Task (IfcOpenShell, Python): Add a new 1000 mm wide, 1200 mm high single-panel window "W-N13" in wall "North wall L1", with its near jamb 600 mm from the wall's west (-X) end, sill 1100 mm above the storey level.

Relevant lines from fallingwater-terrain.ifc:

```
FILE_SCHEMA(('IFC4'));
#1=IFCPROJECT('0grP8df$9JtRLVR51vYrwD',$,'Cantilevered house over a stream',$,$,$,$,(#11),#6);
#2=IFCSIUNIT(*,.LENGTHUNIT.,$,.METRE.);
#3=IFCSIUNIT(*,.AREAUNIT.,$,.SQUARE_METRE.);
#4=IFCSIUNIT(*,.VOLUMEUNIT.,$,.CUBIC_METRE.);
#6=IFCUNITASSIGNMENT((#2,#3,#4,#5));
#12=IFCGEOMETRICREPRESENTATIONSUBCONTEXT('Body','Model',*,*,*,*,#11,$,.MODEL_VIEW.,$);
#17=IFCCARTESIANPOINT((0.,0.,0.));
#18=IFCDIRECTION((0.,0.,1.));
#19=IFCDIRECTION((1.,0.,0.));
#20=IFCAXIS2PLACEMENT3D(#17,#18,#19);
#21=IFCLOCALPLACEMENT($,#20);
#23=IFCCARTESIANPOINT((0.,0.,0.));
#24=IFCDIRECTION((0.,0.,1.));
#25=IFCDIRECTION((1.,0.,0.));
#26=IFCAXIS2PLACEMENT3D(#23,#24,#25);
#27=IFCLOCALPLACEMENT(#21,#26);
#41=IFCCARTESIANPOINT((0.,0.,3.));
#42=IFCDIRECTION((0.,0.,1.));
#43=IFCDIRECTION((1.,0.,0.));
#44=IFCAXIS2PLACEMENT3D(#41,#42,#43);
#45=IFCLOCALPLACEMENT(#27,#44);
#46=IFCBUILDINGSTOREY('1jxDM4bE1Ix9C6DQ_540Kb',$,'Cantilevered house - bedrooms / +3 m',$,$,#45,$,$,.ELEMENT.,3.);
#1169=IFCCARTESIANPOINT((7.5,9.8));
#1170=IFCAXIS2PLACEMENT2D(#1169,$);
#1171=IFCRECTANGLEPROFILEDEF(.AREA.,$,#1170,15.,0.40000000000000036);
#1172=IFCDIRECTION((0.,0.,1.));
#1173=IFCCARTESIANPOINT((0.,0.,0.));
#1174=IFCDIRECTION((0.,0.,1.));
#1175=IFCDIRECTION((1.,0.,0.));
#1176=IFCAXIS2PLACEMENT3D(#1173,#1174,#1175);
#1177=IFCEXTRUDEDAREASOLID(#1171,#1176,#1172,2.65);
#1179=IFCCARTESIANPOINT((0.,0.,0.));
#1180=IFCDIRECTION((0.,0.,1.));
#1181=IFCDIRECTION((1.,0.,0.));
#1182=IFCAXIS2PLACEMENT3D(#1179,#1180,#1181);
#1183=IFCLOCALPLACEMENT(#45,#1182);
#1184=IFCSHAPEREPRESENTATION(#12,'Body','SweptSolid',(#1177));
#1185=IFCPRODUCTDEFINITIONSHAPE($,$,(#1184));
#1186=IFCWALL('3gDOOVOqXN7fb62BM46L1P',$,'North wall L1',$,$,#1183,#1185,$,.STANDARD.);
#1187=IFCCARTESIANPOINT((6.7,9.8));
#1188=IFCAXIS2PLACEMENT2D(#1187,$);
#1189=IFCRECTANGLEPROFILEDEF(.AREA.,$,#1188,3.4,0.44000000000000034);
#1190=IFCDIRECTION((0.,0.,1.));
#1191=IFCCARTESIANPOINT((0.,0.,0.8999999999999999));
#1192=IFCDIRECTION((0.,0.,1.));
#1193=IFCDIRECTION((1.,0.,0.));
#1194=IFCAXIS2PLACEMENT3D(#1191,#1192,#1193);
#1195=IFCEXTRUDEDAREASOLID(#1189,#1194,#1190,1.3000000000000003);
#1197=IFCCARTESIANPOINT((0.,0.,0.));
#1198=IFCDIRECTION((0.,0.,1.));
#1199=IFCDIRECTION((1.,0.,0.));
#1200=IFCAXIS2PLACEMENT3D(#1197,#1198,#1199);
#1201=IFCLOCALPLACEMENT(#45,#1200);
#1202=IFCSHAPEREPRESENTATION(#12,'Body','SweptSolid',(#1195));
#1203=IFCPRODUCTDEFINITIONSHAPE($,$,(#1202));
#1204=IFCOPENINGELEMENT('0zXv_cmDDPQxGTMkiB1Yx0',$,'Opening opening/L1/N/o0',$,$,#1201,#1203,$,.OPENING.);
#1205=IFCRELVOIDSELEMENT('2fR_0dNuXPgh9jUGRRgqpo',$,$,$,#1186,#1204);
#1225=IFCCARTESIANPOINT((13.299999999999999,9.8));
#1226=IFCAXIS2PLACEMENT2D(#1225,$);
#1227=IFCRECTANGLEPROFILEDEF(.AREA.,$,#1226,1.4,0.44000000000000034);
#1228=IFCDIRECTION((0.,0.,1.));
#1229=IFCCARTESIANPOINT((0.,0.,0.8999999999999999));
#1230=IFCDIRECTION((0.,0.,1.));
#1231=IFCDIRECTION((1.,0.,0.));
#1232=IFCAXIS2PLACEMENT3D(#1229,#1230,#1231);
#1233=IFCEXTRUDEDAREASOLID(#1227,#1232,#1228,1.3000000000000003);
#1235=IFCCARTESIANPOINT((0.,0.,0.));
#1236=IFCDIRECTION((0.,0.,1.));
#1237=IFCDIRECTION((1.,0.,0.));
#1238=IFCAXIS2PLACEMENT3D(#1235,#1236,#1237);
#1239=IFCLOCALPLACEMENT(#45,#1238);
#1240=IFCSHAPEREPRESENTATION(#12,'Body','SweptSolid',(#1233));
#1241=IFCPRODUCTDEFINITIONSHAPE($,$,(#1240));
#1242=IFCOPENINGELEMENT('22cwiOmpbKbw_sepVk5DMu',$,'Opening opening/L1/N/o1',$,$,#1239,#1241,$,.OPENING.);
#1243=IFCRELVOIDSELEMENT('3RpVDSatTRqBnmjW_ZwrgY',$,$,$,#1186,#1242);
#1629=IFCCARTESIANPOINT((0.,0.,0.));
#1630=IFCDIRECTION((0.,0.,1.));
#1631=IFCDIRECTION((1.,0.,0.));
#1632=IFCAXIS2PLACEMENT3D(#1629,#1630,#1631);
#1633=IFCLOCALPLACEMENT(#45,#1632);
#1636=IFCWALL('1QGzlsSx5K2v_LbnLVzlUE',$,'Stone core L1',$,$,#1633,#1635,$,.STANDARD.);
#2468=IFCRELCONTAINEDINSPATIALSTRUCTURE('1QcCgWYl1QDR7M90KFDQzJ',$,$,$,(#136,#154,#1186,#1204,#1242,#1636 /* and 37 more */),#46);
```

```python
import numpy as np
import ifcopenshell
import ifcopenshell.api.feature
import ifcopenshell.api.geometry
import ifcopenshell.api.root
import ifcopenshell.api.spatial
import ifcopenshell.geom
import ifcopenshell.util.element
import ifcopenshell.util.placement
import ifcopenshell.util.representation
import ifcopenshell.util.shape
import ifcopenshell.util.unit

model = ifcopenshell.open("fallingwater-terrain.ifc")
unit_scale = ifcopenshell.util.unit.calculate_unit_scale(model)
settings = ifcopenshell.geom.settings()


def volume(element):
    """Net volume in cubic metres, openings subtracted."""
    shape = ifcopenshell.geom.create_shape(settings, element)
    return ifcopenshell.util.shape.get_volume(shape.geometry)


wall = model.by_id(1186)
storey = ifcopenshell.util.element.get_container(wall, ifc_class="IfcBuildingStorey")
context = ifcopenshell.util.representation.get_context(model, "Model", "Body", "MODEL_VIEW")
before = volume(wall)

width, height, from_end, sill = 1, 1.2, 0.6, 1.1  # metres

# The wall runs along its own X axis, and the end named is its -X end.
wall_shape = ifcopenshell.geom.create_shape(settings, wall)
x, y, z = ifcopenshell.util.shape.get_vertices(wall_shape.geometry).T
start = x.min() + from_end
face, thickness = float(y.min()), float(y.max() - y.min())
wall_matrix = ifcopenshell.util.placement.get_local_placement(wall.ObjectPlacement)
level = ifcopenshell.util.placement.get_local_placement(storey.ObjectPlacement)[2, 3]


def in_wall(x, y):
    """Placement at x, y metres in the wall's axes, at sill height."""
    matrix = wall_matrix.copy()
    matrix[:, 3] = wall_matrix @ np.array([x / unit_scale, y / unit_scale, 0.0, 1.0])
    matrix[2, 3] = level + sill / unit_scale
    return matrix


# Opening: a box that overshoots both wall faces by 50 mm.
opening = ifcopenshell.api.root.create_entity(model, ifc_class="IfcOpeningElement", predefined_type="OPENING")
box = ifcopenshell.api.geometry.add_wall_representation(
    model, context=context, length=width, height=height, thickness=thickness + 0.1
)
ifcopenshell.api.geometry.assign_representation(model, product=opening, representation=box)
ifcopenshell.api.geometry.edit_object_placement(model, product=opening, matrix=in_wall(start, face - 0.05), is_si=False)
ifcopenshell.api.feature.add_feature(model, feature=opening, element=wall)

window = ifcopenshell.api.root.create_entity(model, ifc_class="IfcWindow", name="W-N13", predefined_type="WINDOW")
window.OverallWidth, window.OverallHeight = width / unit_scale, height / unit_scale
window.PartitioningType = "SINGLE_PANEL"
body = ifcopenshell.api.geometry.add_window_representation(
    model,
    context=context,
    overall_width=window.OverallWidth,
    overall_height=window.OverallHeight,
    partition_type="SINGLE_PANEL",
)
ifcopenshell.api.geometry.assign_representation(model, product=window, representation=body)
ifcopenshell.api.spatial.assign_container(model, products=[window], relating_structure=storey)
ifcopenshell.api.feature.add_filling(model, opening=opening, element=window)

# Centre the window in the wall's thickness.
ifcopenshell.api.geometry.edit_object_placement(model, product=window, matrix=in_wall(start, face), is_si=False)
window_shape = ifcopenshell.geom.create_shape(settings, window)
depth = ifcopenshell.util.shape.get_vertices(window_shape.geometry)[:, 1]
offset = face + thickness / 2 - (depth.min() + depth.max()) / 2
ifcopenshell.api.geometry.edit_object_placement(model, product=window, matrix=in_wall(start, offset), is_si=False)

after = volume(wall)

print(f"wall volume {before:.3f} -> {after:.3f} m3")

model.write("fallingwater-terrain-out.ifc")
```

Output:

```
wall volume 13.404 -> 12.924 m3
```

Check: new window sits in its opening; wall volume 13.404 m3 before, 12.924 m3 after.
